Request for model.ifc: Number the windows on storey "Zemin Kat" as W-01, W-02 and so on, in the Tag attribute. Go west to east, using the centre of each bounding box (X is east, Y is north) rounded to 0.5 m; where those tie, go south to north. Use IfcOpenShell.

First a look at what the model holds.

```python
import ifcopenshell
import ifcopenshell.util.element
import ifcopenshell.util.placement

model = ifcopenshell.open("model.ifc")
print(model.schema)
storey = next(s for s in model.by_type("IfcBuildingStorey") if s.Name == "Zemin Kat")
windows = [e for e in ifcopenshell.util.element.get_decomposition(storey) if e.is_a("IfcWindow")]
for e in sorted(windows, key=lambda e: e.id()):
    origin = ifcopenshell.util.placement.get_local_placement(e.ObjectPlacement)[:3, 3]
    print(e.id(), e.Tag, e.Name, origin.round(2) + 0.0, sep=" | ")
```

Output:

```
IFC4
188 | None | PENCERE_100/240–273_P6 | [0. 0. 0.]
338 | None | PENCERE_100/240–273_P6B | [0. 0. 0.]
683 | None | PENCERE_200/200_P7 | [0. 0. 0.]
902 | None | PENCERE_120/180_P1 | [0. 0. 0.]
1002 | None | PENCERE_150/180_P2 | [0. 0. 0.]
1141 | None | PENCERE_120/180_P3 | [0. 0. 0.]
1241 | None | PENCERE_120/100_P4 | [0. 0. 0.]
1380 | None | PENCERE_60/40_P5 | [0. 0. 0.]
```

```python
import ifcopenshell
import ifcopenshell.geom
import ifcopenshell.util.element
import ifcopenshell.util.shape

model = ifcopenshell.open("model.ifc")
settings = ifcopenshell.geom.settings()
settings.set("use-world-coords", True)


def centre(element):
    shape = ifcopenshell.geom.create_shape(settings, element)
    return ifcopenshell.util.shape.get_bbox_centroid(shape.geometry)


storey = next(s for s in model.by_type("IfcBuildingStorey") if s.Name == "Zemin Kat")
windows = [e for e in ifcopenshell.util.element.get_decomposition(storey) if e.is_a("IfcWindow")]

# Insertion points can sit at a corner or the storey origin, so sort by the geometry (in metres).
centres = {e: centre(e) for e in windows}
windows.sort(key=lambda e: (round(centres[e][0] / 0.5), centres[e][1]))

for i, e in enumerate(windows, start=1):
    number = f"W-{i:02d}"
    e.Tag = number
    print(e.id(), number)

model.write("model-out.ifc")
```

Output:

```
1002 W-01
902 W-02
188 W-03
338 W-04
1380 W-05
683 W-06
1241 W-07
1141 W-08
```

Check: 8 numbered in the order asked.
